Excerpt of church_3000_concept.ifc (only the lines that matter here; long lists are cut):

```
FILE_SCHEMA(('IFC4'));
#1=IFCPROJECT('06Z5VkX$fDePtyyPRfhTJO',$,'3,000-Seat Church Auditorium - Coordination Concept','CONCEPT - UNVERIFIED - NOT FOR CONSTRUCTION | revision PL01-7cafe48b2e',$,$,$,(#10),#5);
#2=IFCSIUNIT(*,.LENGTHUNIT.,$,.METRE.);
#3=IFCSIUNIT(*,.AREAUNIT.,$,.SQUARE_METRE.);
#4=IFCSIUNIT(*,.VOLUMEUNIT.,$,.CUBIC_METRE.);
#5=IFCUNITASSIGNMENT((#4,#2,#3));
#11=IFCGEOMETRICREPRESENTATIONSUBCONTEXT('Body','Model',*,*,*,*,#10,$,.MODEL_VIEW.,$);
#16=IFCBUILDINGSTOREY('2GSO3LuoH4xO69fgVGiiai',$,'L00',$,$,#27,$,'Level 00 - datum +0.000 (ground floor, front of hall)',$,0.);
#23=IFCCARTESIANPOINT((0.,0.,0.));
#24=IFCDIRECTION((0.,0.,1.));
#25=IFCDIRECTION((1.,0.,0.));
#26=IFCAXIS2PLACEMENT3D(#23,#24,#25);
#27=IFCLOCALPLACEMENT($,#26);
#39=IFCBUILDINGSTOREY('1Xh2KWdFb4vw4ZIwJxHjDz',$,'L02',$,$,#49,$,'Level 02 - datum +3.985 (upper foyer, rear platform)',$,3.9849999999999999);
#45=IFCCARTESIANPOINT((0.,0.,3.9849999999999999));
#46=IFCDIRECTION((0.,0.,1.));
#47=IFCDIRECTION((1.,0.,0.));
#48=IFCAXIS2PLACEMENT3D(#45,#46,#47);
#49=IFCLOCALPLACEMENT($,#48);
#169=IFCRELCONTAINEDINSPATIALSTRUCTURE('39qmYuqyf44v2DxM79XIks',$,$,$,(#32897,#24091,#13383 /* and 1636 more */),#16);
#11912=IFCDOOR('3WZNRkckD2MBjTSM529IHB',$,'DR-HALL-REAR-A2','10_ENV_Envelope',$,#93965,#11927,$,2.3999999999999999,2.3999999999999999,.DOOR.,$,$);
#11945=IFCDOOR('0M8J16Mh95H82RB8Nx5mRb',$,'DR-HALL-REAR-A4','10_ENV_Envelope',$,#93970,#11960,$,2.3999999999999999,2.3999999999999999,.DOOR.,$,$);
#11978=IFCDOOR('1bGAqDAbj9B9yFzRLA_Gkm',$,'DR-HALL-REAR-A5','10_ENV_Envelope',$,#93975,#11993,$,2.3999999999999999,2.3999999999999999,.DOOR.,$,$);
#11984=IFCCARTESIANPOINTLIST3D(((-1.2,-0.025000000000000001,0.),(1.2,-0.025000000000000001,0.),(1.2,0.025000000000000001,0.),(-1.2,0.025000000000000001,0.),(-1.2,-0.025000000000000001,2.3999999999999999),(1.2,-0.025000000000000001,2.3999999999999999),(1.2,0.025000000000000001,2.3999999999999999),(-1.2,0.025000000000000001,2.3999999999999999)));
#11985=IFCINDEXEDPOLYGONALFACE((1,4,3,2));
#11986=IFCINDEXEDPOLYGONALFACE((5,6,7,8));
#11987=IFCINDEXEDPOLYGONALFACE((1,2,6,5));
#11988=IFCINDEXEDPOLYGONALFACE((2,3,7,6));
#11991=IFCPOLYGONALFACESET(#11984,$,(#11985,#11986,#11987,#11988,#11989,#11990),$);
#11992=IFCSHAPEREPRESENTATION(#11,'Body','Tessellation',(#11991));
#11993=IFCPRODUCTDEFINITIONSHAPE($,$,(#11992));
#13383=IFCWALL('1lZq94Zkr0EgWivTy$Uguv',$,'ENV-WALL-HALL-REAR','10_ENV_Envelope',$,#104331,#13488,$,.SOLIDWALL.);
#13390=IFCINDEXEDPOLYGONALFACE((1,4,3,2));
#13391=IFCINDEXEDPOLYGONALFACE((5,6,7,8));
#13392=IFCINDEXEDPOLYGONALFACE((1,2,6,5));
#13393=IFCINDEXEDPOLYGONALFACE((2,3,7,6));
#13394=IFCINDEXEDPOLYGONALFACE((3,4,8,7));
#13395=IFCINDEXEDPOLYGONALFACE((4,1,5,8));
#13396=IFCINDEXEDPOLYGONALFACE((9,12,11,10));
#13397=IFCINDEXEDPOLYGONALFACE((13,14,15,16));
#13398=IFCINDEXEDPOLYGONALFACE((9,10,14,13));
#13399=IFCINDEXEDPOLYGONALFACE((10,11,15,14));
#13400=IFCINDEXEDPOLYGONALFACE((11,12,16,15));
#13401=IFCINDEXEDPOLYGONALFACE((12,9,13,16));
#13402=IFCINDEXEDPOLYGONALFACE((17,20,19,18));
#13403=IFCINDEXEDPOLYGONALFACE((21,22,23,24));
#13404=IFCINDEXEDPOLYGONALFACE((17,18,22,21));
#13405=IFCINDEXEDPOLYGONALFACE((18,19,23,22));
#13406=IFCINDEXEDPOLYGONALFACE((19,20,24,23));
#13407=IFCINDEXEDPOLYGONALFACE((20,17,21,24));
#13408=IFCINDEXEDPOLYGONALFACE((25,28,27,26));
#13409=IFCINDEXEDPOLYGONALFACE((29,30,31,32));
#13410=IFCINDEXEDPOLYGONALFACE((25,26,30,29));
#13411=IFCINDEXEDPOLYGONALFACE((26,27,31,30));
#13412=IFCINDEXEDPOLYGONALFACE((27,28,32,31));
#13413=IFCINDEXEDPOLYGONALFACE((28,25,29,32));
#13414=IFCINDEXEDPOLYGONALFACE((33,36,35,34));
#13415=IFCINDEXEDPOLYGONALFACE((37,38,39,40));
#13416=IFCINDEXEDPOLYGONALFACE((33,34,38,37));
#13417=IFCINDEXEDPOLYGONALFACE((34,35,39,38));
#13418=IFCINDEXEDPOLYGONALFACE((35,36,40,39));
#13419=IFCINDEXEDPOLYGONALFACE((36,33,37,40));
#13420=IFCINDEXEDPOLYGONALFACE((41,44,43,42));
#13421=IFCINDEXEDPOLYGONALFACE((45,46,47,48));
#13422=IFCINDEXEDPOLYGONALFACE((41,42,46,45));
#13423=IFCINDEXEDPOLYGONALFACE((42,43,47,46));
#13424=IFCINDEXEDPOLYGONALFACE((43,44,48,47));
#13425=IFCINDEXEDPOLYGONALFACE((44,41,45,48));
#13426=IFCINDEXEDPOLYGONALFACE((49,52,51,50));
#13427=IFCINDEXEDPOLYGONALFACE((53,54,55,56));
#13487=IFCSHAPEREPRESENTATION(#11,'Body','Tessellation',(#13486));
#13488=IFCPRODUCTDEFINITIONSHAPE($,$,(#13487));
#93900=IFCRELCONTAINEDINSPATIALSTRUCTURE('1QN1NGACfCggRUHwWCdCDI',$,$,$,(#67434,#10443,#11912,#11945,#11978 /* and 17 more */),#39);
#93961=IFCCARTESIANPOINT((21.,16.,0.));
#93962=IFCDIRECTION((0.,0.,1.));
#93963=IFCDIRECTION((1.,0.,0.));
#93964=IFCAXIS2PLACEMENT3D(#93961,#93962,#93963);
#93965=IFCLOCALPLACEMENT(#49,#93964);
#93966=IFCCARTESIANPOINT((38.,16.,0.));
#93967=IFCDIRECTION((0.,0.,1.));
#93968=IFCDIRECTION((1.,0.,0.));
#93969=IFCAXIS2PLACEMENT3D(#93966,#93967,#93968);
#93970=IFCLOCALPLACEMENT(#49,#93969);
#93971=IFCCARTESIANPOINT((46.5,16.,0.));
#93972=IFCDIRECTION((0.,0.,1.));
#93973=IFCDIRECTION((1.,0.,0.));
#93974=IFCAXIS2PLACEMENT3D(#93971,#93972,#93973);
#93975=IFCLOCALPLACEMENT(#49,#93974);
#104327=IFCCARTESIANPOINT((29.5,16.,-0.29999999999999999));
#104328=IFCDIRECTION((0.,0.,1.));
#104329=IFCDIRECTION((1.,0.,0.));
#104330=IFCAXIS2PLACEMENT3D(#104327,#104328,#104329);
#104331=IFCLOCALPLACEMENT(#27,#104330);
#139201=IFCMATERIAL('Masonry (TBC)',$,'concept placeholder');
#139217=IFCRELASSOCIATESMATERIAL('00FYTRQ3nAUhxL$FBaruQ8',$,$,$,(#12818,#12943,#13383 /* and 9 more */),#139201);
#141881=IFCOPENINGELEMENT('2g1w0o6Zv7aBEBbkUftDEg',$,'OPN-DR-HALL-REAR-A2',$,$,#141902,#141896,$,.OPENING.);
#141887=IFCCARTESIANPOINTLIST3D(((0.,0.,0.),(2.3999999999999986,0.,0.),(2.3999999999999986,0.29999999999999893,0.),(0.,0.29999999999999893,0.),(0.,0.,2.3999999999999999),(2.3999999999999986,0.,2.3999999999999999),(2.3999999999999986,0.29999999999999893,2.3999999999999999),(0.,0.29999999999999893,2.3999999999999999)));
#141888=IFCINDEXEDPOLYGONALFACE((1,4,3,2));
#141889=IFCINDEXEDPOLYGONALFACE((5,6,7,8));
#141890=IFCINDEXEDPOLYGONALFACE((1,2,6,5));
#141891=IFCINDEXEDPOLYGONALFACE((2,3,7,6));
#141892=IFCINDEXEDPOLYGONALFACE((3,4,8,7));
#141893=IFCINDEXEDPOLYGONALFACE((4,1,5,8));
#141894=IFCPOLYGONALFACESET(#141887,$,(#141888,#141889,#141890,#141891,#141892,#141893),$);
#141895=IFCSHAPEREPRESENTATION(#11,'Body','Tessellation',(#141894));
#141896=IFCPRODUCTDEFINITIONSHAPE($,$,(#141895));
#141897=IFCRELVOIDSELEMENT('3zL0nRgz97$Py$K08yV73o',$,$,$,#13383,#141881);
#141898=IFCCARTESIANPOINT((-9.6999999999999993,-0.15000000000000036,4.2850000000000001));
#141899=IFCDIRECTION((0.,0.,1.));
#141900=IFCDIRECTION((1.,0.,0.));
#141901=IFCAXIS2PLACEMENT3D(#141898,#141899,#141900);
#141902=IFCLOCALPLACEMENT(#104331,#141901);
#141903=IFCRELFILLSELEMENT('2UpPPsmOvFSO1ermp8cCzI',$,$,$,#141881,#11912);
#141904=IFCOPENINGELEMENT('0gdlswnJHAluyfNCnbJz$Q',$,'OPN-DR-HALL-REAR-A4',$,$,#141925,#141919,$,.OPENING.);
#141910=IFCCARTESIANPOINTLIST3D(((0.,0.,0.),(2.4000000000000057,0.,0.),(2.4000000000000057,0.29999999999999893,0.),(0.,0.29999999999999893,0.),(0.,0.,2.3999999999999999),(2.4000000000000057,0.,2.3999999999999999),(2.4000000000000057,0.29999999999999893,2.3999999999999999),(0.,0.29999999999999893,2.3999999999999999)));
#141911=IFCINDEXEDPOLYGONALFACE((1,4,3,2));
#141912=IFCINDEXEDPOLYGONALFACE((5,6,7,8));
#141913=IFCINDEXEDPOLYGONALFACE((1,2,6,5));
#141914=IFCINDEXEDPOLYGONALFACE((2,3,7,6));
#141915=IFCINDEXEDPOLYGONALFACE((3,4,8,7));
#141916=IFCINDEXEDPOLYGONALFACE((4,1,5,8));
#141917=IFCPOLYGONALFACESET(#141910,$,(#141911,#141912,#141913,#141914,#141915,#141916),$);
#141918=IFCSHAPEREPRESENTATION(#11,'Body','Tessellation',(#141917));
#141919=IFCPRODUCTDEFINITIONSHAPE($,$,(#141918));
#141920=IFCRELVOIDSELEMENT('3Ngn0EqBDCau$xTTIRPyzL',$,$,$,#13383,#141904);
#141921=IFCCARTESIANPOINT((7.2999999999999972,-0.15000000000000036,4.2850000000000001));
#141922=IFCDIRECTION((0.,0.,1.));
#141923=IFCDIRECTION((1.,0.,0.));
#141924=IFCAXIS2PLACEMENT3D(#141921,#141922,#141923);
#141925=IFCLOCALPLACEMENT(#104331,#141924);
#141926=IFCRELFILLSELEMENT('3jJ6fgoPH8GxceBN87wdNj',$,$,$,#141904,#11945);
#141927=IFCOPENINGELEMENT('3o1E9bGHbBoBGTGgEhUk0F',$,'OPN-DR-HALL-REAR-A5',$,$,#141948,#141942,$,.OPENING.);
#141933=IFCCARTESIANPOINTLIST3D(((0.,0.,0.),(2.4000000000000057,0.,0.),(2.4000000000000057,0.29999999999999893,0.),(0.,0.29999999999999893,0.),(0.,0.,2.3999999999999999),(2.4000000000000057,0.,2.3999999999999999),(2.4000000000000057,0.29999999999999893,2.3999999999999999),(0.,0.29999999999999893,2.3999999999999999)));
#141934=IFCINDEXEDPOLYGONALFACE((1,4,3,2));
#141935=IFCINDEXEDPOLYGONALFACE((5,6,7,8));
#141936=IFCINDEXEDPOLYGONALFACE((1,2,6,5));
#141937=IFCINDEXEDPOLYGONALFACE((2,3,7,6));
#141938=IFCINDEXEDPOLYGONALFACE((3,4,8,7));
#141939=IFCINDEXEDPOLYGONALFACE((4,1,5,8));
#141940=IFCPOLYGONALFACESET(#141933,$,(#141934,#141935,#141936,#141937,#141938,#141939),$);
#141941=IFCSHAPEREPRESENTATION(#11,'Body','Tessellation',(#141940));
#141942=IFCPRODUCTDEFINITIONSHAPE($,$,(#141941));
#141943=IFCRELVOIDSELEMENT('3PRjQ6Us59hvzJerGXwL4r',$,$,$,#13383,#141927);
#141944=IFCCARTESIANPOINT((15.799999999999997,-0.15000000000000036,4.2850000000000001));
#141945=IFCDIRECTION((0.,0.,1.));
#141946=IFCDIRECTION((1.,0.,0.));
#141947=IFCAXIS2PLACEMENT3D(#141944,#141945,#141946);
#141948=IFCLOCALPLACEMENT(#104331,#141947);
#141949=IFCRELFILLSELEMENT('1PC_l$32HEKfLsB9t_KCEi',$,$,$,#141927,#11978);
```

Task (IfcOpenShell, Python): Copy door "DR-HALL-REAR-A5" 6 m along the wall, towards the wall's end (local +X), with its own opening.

```python
import ifcopenshell
import ifcopenshell.api.feature
import ifcopenshell.api.geometry
import ifcopenshell.api.root
import ifcopenshell.geom
import ifcopenshell.util.element
import ifcopenshell.util.placement
import ifcopenshell.util.shape

model = ifcopenshell.open("church_3000_concept.ifc")
settings = ifcopenshell.geom.settings()


def volume(element):
    """Net volume in cubic metres, openings subtracted."""
    shape = ifcopenshell.geom.create_shape(settings, element)
    return ifcopenshell.util.shape.get_volume(shape.geometry)


door = model.by_id(11978)
opening = door.FillsVoids[0].RelatingOpeningElement
wall = opening.VoidsElements[0].RelatingBuildingElement
before = volume(wall)
shift = ifcopenshell.util.placement.get_local_placement(wall.ObjectPlacement)[:3, 0] * 6.0

# copy_class copies the void relationship, type, container and properties, but no geometry.
new_opening = ifcopenshell.api.root.copy_class(model, product=opening)
new_opening.Representation = ifcopenshell.util.element.copy_deep(
    model, opening.Representation, exclude=["IfcGeometricRepresentationContext", "IfcRepresentationMap"]
)
new_door = ifcopenshell.api.root.copy_class(model, product=door)
new_door.Representation = ifcopenshell.util.element.copy_deep(
    model, door.Representation, exclude=["IfcGeometricRepresentationContext", "IfcRepresentationMap"]
)
ifcopenshell.api.feature.add_filling(model, opening=new_opening, element=new_door)

for old, new in ((opening, new_opening), (door, new_door)):
    matrix = ifcopenshell.util.placement.get_local_placement(old.ObjectPlacement)
    matrix[:3, 3] += shift
    ifcopenshell.api.geometry.edit_object_placement(model, product=new, matrix=matrix, is_si=False)

after = volume(wall)

print(f"wall volume {before:.3f} -> {after:.3f} m3")

model.write("church_3000_concept-out.ifc")
```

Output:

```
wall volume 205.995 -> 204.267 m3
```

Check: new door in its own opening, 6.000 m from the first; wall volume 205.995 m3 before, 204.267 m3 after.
